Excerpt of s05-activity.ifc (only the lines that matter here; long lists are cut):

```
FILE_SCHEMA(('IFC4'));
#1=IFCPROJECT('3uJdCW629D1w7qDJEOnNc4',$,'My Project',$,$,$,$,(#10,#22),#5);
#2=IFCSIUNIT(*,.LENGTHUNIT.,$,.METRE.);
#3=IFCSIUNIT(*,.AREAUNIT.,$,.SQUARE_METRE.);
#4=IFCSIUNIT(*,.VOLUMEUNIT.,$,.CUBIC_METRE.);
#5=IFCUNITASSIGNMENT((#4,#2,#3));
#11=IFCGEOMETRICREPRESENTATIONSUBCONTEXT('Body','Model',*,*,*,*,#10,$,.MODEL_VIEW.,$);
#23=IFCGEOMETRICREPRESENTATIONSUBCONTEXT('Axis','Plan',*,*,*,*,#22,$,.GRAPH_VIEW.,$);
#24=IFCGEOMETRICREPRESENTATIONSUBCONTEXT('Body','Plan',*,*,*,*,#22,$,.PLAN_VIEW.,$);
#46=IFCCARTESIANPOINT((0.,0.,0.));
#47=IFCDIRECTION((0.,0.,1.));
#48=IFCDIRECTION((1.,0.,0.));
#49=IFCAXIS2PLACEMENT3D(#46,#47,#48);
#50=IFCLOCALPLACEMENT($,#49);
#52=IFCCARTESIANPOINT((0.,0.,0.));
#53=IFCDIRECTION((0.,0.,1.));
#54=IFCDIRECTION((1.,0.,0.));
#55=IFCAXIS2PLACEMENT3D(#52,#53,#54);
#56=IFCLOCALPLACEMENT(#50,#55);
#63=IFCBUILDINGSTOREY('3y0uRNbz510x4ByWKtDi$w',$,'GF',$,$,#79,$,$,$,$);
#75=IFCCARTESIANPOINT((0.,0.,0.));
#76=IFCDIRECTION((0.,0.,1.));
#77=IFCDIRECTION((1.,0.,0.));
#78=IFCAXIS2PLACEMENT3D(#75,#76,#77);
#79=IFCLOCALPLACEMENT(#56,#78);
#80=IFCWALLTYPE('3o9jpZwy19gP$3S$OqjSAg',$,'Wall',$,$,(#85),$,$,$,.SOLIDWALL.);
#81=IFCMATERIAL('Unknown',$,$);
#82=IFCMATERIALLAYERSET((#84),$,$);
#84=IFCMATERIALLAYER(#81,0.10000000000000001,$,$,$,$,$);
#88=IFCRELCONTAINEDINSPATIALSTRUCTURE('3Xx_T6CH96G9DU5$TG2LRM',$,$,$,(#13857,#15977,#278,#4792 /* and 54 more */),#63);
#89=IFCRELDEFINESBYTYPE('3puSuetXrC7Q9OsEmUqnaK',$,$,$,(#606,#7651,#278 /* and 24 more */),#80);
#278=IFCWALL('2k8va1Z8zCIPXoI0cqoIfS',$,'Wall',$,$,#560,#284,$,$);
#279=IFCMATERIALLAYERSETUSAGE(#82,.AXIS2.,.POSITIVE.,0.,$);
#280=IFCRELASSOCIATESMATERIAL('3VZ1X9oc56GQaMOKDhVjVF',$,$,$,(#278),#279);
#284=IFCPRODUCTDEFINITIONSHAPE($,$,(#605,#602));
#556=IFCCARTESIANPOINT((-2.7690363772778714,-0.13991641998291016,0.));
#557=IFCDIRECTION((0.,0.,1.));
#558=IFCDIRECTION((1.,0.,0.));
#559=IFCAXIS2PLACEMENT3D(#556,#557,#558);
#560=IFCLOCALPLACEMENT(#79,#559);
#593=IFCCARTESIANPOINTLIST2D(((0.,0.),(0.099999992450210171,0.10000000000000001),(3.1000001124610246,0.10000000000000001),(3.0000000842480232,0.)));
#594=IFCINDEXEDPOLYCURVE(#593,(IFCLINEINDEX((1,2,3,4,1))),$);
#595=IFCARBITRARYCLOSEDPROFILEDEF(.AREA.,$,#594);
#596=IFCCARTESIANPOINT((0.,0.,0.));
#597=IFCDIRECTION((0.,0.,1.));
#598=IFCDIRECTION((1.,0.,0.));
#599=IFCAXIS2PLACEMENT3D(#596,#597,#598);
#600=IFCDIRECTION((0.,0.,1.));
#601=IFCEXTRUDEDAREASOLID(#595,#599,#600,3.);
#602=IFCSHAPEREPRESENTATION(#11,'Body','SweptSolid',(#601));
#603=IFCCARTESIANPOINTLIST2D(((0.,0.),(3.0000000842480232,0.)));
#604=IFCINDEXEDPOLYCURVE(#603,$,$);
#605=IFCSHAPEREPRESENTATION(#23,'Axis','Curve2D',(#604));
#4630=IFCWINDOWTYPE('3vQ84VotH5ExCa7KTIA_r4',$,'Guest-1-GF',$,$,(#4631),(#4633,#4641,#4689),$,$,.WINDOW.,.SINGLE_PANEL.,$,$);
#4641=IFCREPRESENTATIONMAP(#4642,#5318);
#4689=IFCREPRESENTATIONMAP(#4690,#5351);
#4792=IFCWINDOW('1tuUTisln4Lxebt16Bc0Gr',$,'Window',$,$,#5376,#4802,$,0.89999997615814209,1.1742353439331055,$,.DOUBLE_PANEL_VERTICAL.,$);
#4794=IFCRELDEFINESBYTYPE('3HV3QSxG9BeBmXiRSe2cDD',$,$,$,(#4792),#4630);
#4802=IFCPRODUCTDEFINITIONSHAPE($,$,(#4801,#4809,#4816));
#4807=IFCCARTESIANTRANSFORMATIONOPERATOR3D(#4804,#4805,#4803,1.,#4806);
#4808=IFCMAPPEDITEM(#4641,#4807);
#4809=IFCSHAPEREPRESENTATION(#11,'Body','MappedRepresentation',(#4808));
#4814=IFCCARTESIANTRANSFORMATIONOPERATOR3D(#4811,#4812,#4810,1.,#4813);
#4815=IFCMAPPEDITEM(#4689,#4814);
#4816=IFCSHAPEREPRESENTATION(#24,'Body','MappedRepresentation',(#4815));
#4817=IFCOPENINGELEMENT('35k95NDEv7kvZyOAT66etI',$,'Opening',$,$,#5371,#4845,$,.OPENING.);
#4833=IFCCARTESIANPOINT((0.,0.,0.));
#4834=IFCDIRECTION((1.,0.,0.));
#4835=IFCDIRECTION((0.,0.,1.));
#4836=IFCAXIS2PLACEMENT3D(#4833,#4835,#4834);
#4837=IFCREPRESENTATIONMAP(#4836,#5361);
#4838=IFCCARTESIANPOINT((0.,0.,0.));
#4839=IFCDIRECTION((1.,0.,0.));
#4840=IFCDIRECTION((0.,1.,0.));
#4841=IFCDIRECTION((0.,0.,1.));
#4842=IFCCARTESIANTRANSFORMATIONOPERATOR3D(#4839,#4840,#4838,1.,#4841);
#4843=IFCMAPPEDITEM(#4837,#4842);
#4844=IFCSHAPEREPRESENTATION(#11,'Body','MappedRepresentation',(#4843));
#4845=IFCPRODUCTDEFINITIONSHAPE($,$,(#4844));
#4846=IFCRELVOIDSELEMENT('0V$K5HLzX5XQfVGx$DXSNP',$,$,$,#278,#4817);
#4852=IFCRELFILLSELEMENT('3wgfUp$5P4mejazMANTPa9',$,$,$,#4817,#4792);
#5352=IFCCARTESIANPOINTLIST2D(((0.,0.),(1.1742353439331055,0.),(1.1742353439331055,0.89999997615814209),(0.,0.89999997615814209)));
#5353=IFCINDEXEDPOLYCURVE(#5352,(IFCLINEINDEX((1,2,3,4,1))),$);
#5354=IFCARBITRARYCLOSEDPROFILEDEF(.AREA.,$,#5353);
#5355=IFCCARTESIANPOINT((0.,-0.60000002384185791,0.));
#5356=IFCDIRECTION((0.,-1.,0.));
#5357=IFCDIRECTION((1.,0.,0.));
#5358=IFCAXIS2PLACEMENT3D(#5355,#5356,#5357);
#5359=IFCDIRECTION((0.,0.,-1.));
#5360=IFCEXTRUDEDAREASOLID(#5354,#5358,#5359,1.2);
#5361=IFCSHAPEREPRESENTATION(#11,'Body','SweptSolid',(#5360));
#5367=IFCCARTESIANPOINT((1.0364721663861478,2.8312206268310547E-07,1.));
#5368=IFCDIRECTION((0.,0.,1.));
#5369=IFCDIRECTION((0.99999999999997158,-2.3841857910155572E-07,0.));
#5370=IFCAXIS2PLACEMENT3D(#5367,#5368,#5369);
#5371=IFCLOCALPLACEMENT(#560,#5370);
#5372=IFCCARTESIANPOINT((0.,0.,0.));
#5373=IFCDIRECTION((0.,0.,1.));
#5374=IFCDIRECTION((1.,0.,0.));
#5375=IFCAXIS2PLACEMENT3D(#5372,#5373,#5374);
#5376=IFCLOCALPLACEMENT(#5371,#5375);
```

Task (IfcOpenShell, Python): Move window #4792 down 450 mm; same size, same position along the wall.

```python
import numpy as np
import ifcopenshell
import ifcopenshell.api.geometry
import ifcopenshell.util.placement
import ifcopenshell.util.unit

model = ifcopenshell.open("s05-activity.ifc")
unit_scale = ifcopenshell.util.unit.calculate_unit_scale(model)

window = model.by_id(4792)
opening = window.FillsVoids[0].RelatingOpeningElement
dz = -0.45 / unit_scale

shift = np.array([0.0, 0.0, dz])
# The window is placed relative to its opening, so it follows when the opening moves.
matrix = ifcopenshell.util.placement.get_local_placement(opening.ObjectPlacement)
matrix[:3, 3] += shift
ifcopenshell.api.geometry.edit_object_placement(
    model, product=opening, matrix=matrix, is_si=False, should_transform_children=True
)

print(f"moved by {dz * unit_scale:+.3f} m")

model.write("s05-activity_v2.ifc")
```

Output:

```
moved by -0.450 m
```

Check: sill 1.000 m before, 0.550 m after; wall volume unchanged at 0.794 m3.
